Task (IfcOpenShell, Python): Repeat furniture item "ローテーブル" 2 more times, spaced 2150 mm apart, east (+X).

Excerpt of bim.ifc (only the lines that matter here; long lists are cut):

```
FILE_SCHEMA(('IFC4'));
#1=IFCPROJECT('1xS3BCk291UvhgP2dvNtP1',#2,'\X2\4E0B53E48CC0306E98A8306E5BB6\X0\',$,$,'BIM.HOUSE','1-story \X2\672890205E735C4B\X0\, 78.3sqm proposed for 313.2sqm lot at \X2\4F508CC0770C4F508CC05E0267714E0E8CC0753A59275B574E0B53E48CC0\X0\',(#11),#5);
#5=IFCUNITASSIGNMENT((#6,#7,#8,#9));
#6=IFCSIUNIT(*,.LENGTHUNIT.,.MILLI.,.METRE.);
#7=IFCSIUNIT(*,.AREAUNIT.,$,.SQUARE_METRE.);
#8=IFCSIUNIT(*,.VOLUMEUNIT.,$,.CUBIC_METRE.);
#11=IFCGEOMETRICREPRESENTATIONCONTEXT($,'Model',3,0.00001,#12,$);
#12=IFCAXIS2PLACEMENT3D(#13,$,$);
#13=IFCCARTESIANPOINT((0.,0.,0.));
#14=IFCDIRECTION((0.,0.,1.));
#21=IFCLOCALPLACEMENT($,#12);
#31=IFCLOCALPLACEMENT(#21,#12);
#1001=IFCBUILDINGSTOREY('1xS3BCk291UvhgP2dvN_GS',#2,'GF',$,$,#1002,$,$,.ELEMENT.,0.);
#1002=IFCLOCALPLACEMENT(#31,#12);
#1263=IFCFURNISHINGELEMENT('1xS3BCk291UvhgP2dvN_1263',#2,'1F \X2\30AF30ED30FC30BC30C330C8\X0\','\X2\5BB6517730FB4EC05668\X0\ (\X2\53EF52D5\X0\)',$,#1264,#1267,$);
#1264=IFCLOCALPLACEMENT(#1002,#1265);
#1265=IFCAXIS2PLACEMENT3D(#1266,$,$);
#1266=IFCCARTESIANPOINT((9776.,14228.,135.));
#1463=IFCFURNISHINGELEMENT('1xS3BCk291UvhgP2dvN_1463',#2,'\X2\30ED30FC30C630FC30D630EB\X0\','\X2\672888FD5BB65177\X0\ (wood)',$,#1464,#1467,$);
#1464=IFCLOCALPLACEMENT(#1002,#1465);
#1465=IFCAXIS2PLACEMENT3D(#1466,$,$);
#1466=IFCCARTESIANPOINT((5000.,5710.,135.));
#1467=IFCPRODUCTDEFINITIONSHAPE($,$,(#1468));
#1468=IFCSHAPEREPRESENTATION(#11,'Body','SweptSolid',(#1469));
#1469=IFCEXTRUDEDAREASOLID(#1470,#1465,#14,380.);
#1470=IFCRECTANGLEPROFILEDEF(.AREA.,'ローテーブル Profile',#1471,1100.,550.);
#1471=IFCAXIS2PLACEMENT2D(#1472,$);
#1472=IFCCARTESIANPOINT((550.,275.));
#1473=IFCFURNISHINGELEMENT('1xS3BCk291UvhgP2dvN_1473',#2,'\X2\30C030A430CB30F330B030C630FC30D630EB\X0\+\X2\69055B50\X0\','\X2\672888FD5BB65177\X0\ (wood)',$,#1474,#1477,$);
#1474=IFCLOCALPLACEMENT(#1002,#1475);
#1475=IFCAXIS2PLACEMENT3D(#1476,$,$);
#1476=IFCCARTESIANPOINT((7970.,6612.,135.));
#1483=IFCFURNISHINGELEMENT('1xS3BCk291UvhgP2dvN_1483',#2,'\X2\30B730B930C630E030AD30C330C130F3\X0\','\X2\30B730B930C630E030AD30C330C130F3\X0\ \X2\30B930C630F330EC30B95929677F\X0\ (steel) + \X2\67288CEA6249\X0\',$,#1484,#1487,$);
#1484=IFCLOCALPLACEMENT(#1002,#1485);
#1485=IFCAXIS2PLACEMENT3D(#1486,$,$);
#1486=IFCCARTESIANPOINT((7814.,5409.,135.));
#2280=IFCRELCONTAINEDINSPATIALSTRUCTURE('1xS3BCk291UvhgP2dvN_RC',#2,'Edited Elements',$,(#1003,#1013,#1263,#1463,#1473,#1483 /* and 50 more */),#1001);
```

```python
import numpy as np
import ifcopenshell
import ifcopenshell.api.geometry
import ifcopenshell.api.root
import ifcopenshell.util.element
import ifcopenshell.util.placement

model = ifcopenshell.open("bim.ifc")


def reuse_history(source, copy):
    """copy_class also copies each property set's owner history, people and application; keep the originals."""
    for rel in copy.IsDefinedBy:
        if rel.is_a("IfcRelDefinesByProperties") and (history := rel.RelatingPropertyDefinition.OwnerHistory):
            rel.RelatingPropertyDefinition.OwnerHistory = source.OwnerHistory
            ifcopenshell.util.element.remove_deep2(model, history)


source = model.by_id(1463)
base = ifcopenshell.util.placement.get_local_placement(source.ObjectPlacement)
step = np.array([1.0, 0.0, 0.0]) * 2150.0

for i in range(1, 3):
    copy = ifcopenshell.api.root.copy_class(model, product=source)
    copy.Representation = ifcopenshell.util.element.copy_deep(
        model, source.Representation, exclude=["IfcGeometricRepresentationContext", "IfcRepresentationMap"]
    )
    reuse_history(source, copy)
    matrix = base.copy()
    matrix[:3, 3] += i * step
    print("added at", matrix[:3, 3].round(3) + 0.0)
    ifcopenshell.api.geometry.edit_object_placement(model, product=copy, matrix=matrix, is_si=False)

model.write("bim_v2.ifc")
```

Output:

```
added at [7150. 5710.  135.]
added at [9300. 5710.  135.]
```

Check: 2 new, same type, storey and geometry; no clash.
